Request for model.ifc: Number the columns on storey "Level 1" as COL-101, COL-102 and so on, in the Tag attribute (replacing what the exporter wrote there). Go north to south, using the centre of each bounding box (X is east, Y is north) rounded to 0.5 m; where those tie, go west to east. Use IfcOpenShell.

First a look at what the model holds.

```python
import ifcopenshell
import ifcopenshell.util.element
import ifcopenshell.util.placement

model = ifcopenshell.open("model.ifc")
print(model.schema)
storey = next(s for s in model.by_type("IfcBuildingStorey") if s.Name == "Level 1")
columns = [e for e in ifcopenshell.util.element.get_decomposition(storey) if e.is_a("IfcColumn")]
for e in sorted(columns, key=lambda e: e.id()):
    origin = ifcopenshell.util.placement.get_local_placement(e.ObjectPlacement)[:3, 3]
    print(e.id(), e.Tag, e.Name, origin.round(2) + 0.0, sep=" | ")
```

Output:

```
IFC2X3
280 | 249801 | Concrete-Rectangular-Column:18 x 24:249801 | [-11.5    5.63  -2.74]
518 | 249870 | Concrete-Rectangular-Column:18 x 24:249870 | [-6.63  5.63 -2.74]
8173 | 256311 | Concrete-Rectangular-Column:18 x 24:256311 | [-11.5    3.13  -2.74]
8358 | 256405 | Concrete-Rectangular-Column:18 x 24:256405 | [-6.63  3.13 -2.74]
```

```python
import ifcopenshell
import ifcopenshell.geom
import ifcopenshell.util.element
import ifcopenshell.util.shape

model = ifcopenshell.open("model.ifc")
settings = ifcopenshell.geom.settings()
settings.set("use-world-coords", True)


def centre(element):
    shape = ifcopenshell.geom.create_shape(settings, element)
    return ifcopenshell.util.shape.get_bbox_centroid(shape.geometry)


storey = next(s for s in model.by_type("IfcBuildingStorey") if s.Name == "Level 1")
columns = [e for e in ifcopenshell.util.element.get_decomposition(storey) if e.is_a("IfcColumn")]

# Insertion points can sit at a corner or the storey origin, so sort by the geometry (in metres).
centres = {e: centre(e) for e in columns}
columns.sort(key=lambda e: (-round(centres[e][1] / 0.5), centres[e][0]))

for i, e in enumerate(columns, start=1):
    number = f"COL-1{i:02d}"
    e.Tag = number
    print(e.id(), number)

model.write("model_v2.ifc")
```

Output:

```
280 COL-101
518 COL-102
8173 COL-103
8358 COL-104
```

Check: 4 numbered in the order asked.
